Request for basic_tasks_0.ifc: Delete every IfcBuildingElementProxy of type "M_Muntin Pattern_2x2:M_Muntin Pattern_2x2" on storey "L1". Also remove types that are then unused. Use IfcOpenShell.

First a look at what the model holds.

```python
import ifcopenshell
import ifcopenshell.util.element

model = ifcopenshell.open("basic_tasks_0.ifc")
print(model.schema)
storey = next(s for s in model.by_type("IfcBuildingStorey") if s.Name == "L1")
proxies = [e for e in ifcopenshell.util.element.get_decomposition(storey) if e.is_a("IfcBuildingElementProxy")]
seen = {}
for e in proxies:
    element_type = ifcopenshell.util.element.get_type(e)
    name = element_type.Name if element_type not in (None, e) else None
    seen[name] = seen.get(name, 0) + 1
for name, count in sorted(seen.items(), key=str):
    print(count, "x", name)
```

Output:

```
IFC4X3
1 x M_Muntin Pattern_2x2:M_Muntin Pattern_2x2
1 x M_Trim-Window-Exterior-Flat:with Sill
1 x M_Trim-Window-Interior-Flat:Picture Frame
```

```python
import ifcopenshell
import ifcopenshell.api.root
import ifcopenshell.util.element

model = ifcopenshell.open("basic_tasks_0.ifc")

storey = next(s for s in model.by_type("IfcBuildingStorey") if s.Name == "L1")
proxies = [e for e in ifcopenshell.util.element.get_decomposition(storey) if e.is_a("IfcBuildingElementProxy")]
targets = [e for e in proxies if (t := ifcopenshell.util.element.get_type(e)) not in (None, e) and t.Name == "M_Muntin Pattern_2x2:M_Muntin Pattern_2x2"]
types = {ifcopenshell.util.element.get_type(e) for e in targets} - {None, *targets}

for e in targets:
    ifcopenshell.api.root.remove_product(model, product=e)
print(len(targets), "removed")

unused = [t for t in types if not ifcopenshell.util.element.get_types(t)]
for t in unused:
    ifcopenshell.api.root.remove_product(model, product=t)
print(len(unused), "unused types removed")

model.write("basic_tasks_0_edited.ifc")
```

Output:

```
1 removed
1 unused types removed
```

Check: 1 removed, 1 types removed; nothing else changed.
